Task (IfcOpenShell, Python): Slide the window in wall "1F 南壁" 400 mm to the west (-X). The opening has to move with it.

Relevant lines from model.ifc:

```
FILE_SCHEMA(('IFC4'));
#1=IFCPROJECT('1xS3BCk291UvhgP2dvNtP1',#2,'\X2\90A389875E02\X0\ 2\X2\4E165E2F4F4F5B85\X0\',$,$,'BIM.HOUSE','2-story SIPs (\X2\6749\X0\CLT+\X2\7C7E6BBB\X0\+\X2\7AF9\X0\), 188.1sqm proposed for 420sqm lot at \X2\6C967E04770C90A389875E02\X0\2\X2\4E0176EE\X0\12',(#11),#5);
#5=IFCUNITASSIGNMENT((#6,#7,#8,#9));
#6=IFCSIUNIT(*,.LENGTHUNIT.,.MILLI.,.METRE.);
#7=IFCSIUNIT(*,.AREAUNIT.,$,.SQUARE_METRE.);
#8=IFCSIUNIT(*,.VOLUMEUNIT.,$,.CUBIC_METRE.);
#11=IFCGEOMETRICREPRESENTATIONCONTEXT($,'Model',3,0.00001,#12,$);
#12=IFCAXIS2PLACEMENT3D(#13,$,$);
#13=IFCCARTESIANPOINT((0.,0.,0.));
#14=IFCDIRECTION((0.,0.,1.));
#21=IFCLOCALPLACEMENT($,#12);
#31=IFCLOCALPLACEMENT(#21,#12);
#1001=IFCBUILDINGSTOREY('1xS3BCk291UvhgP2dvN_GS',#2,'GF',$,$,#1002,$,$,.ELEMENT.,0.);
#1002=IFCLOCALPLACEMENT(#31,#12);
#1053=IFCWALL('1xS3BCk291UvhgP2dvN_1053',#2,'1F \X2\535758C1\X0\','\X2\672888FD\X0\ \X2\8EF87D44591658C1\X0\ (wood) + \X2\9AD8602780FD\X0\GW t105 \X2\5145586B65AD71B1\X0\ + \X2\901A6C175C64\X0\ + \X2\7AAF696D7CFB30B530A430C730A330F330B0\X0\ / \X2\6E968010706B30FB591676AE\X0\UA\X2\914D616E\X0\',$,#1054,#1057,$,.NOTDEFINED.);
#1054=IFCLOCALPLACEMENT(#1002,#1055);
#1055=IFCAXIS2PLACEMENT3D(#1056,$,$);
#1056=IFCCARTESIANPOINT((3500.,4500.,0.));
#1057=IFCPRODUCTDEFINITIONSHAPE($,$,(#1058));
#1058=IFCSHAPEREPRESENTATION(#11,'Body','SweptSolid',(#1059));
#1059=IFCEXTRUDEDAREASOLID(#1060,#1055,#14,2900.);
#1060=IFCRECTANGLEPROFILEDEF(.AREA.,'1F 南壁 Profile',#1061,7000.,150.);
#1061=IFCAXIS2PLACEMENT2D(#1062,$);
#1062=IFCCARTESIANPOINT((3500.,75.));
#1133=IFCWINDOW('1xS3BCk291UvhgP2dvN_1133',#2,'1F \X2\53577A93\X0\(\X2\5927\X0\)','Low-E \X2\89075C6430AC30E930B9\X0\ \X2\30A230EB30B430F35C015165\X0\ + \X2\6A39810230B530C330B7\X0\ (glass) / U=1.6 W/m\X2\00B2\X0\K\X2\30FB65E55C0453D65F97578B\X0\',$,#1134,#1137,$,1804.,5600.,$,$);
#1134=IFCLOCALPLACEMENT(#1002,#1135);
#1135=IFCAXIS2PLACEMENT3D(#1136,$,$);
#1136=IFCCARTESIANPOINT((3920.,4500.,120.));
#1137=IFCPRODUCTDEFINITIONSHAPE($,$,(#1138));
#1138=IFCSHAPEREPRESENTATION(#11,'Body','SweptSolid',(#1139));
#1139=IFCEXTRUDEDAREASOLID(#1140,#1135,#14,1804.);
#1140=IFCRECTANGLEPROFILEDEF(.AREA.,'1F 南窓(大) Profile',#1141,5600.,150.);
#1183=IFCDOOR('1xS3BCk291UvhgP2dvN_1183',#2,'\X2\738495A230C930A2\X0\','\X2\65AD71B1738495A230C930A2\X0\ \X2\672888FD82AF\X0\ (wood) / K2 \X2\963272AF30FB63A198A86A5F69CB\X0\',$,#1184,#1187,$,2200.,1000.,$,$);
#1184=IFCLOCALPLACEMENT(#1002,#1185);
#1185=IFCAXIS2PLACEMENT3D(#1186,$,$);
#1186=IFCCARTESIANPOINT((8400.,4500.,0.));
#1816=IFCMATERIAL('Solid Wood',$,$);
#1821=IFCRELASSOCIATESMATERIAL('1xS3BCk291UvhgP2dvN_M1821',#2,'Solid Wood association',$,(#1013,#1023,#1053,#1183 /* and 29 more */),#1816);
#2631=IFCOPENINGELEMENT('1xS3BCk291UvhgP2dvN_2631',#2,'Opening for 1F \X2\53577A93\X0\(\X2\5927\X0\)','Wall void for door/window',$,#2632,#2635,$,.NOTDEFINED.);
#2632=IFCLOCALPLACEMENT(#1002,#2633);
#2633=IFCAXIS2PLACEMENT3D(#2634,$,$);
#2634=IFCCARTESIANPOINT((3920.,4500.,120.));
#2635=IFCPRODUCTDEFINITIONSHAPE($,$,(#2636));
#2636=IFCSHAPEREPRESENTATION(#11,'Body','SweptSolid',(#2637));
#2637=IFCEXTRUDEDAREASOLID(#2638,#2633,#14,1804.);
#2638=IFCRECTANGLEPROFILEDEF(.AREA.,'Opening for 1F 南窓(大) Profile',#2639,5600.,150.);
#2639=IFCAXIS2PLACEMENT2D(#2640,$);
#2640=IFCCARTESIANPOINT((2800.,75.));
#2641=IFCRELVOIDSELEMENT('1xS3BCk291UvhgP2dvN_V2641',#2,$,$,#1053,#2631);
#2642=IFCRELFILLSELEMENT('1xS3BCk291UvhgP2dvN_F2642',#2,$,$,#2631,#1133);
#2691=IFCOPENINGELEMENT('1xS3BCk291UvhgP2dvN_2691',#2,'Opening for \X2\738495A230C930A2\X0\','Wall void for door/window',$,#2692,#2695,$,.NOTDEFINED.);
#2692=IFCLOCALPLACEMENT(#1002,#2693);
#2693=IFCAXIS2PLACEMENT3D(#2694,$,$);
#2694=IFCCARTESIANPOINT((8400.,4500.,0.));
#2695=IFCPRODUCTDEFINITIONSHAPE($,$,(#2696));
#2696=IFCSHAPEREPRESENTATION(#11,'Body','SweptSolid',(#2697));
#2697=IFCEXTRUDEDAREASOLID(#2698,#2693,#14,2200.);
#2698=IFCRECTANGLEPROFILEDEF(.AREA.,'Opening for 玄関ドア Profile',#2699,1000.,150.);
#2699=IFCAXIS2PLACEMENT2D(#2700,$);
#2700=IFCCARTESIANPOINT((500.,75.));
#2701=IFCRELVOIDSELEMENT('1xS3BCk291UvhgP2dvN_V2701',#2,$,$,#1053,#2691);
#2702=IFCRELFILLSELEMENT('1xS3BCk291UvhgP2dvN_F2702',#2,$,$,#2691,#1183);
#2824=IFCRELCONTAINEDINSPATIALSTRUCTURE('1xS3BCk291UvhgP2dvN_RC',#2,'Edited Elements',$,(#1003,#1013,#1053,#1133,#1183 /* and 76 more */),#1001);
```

```python
import ifcopenshell
import ifcopenshell.api.geometry
import ifcopenshell.util.placement
import ifcopenshell.util.unit

model = ifcopenshell.open("model.ifc")
unit_scale = ifcopenshell.util.unit.calculate_unit_scale(model)

window = model.by_id(1133)
opening = window.FillsVoids[0].RelatingOpeningElement
wall = opening.VoidsElements[0].RelatingBuildingElement

wall_matrix = ifcopenshell.util.placement.get_local_placement(wall.ObjectPlacement)
shift = wall_matrix[:3, 0] * -0.4 / unit_scale
before = ifcopenshell.util.placement.get_local_placement(window.ObjectPlacement)[:3, 3].copy()

# The window is not placed relative to its opening, so move both.
for product in (opening, window):
    matrix = ifcopenshell.util.placement.get_local_placement(product.ObjectPlacement)
    matrix[:3, 3] += shift
    ifcopenshell.api.geometry.edit_object_placement(model, product=product, matrix=matrix, is_si=False)

after = ifcopenshell.util.placement.get_local_placement(window.ObjectPlacement)[:3, 3]
print("window moved by", (after - before).round(3) + 0.0)

model.write("model_rev.ifc")
```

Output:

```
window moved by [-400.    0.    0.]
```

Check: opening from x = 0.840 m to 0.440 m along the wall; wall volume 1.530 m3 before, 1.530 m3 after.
